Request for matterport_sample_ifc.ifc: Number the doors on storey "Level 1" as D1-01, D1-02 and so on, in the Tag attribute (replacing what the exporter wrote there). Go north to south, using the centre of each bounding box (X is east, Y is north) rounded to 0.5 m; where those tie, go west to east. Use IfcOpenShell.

First a look at what the model holds.

```python
import ifcopenshell
import ifcopenshell.util.element
import ifcopenshell.util.placement

model = ifcopenshell.open("matterport_sample_ifc.ifc")
print(model.schema)
storey = next(s for s in model.by_type("IfcBuildingStorey") if s.Name == "Level 1")
doors = [e for e in ifcopenshell.util.element.get_decomposition(storey) if e.is_a("IfcDoor")]
for e in sorted(doors, key=lambda e: e.id()):
    origin = ifcopenshell.util.placement.get_local_placement(e.ObjectPlacement)[:3, 3]
    print(e.id(), e.Tag, e.Name, origin.round(2) + 0.0, sep=" | ")
```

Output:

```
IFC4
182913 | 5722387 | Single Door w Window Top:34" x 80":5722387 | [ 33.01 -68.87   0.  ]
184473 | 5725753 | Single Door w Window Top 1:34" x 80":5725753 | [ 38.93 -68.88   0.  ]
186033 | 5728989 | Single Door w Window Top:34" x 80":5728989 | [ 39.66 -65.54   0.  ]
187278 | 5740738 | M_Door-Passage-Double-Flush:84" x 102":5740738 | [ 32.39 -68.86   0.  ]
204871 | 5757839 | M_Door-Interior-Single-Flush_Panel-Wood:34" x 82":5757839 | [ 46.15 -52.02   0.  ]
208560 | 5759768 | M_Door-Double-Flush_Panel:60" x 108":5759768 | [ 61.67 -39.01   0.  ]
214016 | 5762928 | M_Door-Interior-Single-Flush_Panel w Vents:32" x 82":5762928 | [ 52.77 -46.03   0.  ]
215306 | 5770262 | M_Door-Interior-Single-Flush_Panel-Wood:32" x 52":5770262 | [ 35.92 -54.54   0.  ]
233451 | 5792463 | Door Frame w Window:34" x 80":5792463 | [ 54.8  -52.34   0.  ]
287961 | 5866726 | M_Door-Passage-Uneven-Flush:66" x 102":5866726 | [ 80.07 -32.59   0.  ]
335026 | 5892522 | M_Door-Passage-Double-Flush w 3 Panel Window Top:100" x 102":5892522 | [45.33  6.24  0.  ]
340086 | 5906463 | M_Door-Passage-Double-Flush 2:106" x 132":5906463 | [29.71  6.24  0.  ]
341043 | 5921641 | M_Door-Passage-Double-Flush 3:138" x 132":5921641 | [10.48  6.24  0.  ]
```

```python
import ifcopenshell
import ifcopenshell.geom
import ifcopenshell.util.element
import ifcopenshell.util.shape

model = ifcopenshell.open("matterport_sample_ifc.ifc")
settings = ifcopenshell.geom.settings()
settings.set("use-world-coords", True)


def centre(element):
    shape = ifcopenshell.geom.create_shape(settings, element)
    return ifcopenshell.util.shape.get_bbox_centroid(shape.geometry)


storey = next(s for s in model.by_type("IfcBuildingStorey") if s.Name == "Level 1")
doors = [e for e in ifcopenshell.util.element.get_decomposition(storey) if e.is_a("IfcDoor")]

# Insertion points can sit at a corner or the storey origin, so sort by the geometry (in metres).
centres = {e: centre(e) for e in doors}
doors.sort(key=lambda e: (-round(centres[e][1] / 0.5), centres[e][0]))

for i, e in enumerate(doors, start=1):
    number = f"D1-{i:02d}"
    e.Tag = number
    print(e.id(), number)

model.write("matterport_sample_ifc_updated.ifc")
```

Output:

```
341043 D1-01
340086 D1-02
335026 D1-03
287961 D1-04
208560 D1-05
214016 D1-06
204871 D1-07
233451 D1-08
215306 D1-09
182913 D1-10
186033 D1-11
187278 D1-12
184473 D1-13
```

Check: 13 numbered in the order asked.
